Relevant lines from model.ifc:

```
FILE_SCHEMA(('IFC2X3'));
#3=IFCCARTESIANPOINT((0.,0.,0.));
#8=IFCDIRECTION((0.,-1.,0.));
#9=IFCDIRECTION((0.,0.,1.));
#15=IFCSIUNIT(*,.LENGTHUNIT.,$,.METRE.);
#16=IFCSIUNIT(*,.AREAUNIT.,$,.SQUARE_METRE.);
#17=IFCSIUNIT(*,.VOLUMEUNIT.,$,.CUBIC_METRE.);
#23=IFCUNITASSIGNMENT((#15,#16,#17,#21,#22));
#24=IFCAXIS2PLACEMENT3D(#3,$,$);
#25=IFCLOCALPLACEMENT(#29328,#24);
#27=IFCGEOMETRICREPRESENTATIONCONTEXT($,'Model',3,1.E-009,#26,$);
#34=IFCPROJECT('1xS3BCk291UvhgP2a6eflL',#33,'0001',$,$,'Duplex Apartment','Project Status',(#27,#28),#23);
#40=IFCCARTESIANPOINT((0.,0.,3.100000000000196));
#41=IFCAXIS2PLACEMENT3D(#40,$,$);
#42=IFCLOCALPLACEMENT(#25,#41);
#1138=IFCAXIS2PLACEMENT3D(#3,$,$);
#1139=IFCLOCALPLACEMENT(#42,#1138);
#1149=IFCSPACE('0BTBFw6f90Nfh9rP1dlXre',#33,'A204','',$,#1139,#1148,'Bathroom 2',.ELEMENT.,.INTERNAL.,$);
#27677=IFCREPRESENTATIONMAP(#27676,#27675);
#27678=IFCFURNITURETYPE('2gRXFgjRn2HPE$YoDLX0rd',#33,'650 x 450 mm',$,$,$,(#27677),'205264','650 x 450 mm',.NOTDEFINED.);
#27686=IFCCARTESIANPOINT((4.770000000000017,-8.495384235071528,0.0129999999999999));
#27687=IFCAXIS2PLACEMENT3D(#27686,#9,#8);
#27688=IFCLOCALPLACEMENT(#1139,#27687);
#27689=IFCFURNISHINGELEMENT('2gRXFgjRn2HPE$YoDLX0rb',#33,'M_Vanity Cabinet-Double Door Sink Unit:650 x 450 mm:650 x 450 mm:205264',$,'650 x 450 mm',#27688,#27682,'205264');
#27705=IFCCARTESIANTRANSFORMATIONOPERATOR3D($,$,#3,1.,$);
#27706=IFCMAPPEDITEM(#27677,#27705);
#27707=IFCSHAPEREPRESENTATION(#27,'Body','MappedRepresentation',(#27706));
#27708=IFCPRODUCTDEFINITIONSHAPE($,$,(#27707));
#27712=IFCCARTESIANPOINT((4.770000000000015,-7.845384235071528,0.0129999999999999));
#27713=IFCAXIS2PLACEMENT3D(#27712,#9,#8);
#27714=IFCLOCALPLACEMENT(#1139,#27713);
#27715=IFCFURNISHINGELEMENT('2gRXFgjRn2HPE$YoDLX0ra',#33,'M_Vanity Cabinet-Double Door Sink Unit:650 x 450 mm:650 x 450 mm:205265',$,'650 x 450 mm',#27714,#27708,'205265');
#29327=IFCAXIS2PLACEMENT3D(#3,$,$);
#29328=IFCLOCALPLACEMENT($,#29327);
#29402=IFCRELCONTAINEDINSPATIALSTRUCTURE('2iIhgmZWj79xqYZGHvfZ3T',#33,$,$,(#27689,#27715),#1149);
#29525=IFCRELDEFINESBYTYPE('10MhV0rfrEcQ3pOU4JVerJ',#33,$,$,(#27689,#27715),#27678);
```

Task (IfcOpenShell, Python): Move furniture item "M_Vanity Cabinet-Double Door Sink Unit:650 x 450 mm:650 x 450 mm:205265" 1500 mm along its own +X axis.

```python
import ifcopenshell
import ifcopenshell.api.geometry
import ifcopenshell.util.placement
import ifcopenshell.util.unit

model = ifcopenshell.open("model.ifc")
unit_scale = ifcopenshell.util.unit.calculate_unit_scale(model)

item = model.by_guid("2gRXFgjRn2HPE$YoDLX0ra")
matrix = ifcopenshell.util.placement.get_local_placement(item.ObjectPlacement)
matrix[:3, 3] += matrix[:3, 0] * 1.5 / unit_scale
ifcopenshell.api.geometry.edit_object_placement(model, product=item, matrix=matrix, is_si=False)

print(ifcopenshell.util.placement.get_local_placement(item.ObjectPlacement).round(3) + 0.0)

model.write("model_edited.ifc")
```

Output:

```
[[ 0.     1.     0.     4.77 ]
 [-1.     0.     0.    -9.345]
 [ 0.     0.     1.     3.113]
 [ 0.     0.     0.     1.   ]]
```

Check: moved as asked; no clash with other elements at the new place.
